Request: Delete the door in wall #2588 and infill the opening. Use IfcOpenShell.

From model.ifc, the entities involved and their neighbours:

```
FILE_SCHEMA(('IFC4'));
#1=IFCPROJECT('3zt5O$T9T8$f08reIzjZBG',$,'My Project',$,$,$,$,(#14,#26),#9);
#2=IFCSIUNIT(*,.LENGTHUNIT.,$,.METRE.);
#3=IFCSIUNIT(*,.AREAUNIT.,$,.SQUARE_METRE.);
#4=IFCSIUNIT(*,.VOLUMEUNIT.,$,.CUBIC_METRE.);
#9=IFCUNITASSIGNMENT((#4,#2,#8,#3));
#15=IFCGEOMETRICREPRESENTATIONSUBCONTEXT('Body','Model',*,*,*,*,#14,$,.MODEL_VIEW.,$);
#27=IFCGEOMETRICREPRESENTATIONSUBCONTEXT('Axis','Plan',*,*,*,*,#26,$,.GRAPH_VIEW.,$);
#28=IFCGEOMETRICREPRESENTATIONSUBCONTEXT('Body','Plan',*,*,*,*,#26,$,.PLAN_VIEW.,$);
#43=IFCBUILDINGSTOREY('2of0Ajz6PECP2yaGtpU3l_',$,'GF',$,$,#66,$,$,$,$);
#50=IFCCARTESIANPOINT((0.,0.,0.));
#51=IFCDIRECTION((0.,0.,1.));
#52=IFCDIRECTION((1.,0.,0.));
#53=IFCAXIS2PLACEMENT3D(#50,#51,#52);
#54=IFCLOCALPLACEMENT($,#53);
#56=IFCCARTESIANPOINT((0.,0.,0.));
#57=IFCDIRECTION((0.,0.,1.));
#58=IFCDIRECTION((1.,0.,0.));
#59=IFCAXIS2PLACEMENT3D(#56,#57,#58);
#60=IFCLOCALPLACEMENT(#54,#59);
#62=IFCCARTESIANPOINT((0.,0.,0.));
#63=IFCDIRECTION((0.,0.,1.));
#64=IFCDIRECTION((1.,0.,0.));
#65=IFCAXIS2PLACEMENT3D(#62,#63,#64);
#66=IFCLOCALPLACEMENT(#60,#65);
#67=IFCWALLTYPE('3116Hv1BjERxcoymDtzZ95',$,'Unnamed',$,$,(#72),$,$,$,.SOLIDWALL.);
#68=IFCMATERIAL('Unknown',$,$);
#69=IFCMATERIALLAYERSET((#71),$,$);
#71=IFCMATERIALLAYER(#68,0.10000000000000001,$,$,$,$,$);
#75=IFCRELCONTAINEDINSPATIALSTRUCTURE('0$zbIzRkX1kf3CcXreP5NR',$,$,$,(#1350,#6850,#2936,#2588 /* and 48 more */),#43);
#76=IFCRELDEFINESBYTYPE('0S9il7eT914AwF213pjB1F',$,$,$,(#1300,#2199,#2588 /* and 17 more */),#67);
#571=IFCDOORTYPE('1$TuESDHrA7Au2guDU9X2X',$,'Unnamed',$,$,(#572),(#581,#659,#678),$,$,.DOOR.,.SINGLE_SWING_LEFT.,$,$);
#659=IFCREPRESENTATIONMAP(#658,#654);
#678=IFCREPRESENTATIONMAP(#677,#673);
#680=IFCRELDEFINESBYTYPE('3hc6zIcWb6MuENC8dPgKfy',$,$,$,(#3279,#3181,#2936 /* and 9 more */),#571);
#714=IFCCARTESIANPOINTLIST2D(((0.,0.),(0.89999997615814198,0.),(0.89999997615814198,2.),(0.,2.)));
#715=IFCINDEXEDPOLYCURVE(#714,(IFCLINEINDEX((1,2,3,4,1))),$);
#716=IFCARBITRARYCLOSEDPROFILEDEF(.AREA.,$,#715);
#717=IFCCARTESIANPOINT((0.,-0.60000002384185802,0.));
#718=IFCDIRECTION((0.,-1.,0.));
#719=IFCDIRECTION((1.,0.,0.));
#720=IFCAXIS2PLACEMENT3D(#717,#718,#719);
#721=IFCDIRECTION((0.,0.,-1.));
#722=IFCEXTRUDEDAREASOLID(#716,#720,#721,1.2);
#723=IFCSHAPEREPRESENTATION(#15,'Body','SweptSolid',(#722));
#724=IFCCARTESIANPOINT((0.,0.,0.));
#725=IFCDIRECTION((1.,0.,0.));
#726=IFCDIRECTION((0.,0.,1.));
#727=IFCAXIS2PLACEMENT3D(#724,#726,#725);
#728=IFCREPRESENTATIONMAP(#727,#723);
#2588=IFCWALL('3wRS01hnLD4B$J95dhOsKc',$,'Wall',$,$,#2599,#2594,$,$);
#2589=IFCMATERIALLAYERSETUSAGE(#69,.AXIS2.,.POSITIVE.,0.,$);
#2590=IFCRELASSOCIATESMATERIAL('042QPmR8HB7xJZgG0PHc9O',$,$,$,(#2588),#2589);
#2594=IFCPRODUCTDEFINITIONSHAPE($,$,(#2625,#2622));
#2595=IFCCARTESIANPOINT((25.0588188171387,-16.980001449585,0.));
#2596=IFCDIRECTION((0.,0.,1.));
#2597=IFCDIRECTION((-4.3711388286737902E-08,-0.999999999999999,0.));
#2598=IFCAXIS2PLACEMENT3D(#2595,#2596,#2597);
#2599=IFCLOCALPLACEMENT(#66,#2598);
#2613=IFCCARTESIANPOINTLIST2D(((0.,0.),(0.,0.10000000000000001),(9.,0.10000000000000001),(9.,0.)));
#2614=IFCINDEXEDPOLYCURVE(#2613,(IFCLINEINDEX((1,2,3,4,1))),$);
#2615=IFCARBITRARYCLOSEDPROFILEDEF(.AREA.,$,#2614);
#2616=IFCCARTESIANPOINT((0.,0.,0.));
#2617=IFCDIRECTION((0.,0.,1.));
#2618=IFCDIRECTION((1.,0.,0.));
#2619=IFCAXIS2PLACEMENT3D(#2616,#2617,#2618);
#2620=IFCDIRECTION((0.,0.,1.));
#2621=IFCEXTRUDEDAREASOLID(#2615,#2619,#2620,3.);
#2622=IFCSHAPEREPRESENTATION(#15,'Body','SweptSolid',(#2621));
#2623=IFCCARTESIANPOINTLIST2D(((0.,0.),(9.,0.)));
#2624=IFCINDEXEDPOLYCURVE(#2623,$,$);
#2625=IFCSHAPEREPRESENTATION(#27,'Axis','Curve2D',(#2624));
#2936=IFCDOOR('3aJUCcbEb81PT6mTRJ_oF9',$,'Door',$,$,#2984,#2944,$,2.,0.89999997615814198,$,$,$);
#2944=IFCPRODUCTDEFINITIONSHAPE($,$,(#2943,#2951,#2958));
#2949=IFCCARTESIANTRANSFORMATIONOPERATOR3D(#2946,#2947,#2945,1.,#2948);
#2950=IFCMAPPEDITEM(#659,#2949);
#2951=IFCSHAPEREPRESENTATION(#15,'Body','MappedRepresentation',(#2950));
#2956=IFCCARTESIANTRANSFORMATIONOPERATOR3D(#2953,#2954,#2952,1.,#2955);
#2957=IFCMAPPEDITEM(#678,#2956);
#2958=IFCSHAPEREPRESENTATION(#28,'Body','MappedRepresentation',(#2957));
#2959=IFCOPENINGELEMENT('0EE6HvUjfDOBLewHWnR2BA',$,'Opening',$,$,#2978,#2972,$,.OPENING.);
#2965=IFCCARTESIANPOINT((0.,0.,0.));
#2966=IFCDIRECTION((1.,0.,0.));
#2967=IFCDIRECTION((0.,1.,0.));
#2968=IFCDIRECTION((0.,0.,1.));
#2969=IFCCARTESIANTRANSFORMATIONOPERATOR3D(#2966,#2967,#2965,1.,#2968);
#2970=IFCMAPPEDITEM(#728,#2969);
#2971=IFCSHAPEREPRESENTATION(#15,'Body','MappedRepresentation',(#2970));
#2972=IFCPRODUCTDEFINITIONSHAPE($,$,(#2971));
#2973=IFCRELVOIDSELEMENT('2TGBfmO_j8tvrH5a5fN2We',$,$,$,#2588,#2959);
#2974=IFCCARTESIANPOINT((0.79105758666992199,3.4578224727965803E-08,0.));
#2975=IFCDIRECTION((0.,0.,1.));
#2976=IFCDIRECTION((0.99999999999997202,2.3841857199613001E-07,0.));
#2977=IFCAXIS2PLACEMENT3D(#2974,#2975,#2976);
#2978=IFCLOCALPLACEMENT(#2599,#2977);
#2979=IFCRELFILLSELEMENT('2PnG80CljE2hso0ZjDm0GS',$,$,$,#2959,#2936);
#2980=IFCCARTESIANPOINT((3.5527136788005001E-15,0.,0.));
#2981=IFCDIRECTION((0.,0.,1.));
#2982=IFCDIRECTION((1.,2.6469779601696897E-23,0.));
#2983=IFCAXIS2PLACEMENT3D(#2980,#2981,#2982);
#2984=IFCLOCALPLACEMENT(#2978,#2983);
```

```python
import ifcopenshell
import ifcopenshell.api.feature
import ifcopenshell.api.root
import ifcopenshell.geom
import ifcopenshell.util.shape

model = ifcopenshell.open("model.ifc")
settings = ifcopenshell.geom.settings()


def volume(element):
    """Net volume in cubic metres, openings subtracted."""
    shape = ifcopenshell.geom.create_shape(settings, element)
    return ifcopenshell.util.shape.get_volume(shape.geometry)


door = model.by_id(2936)
opening = door.FillsVoids[0].RelatingOpeningElement
wall = opening.VoidsElements[0].RelatingBuildingElement
before = volume(wall)

ifcopenshell.api.root.remove_product(model, product=door)
ifcopenshell.api.feature.remove_feature(model, feature=opening)

after = volume(wall)

print(f"wall volume {before:.3f} -> {after:.3f} m3")

model.write("model_updated.ifc")
```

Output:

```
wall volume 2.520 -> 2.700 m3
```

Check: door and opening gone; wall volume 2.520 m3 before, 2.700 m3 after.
